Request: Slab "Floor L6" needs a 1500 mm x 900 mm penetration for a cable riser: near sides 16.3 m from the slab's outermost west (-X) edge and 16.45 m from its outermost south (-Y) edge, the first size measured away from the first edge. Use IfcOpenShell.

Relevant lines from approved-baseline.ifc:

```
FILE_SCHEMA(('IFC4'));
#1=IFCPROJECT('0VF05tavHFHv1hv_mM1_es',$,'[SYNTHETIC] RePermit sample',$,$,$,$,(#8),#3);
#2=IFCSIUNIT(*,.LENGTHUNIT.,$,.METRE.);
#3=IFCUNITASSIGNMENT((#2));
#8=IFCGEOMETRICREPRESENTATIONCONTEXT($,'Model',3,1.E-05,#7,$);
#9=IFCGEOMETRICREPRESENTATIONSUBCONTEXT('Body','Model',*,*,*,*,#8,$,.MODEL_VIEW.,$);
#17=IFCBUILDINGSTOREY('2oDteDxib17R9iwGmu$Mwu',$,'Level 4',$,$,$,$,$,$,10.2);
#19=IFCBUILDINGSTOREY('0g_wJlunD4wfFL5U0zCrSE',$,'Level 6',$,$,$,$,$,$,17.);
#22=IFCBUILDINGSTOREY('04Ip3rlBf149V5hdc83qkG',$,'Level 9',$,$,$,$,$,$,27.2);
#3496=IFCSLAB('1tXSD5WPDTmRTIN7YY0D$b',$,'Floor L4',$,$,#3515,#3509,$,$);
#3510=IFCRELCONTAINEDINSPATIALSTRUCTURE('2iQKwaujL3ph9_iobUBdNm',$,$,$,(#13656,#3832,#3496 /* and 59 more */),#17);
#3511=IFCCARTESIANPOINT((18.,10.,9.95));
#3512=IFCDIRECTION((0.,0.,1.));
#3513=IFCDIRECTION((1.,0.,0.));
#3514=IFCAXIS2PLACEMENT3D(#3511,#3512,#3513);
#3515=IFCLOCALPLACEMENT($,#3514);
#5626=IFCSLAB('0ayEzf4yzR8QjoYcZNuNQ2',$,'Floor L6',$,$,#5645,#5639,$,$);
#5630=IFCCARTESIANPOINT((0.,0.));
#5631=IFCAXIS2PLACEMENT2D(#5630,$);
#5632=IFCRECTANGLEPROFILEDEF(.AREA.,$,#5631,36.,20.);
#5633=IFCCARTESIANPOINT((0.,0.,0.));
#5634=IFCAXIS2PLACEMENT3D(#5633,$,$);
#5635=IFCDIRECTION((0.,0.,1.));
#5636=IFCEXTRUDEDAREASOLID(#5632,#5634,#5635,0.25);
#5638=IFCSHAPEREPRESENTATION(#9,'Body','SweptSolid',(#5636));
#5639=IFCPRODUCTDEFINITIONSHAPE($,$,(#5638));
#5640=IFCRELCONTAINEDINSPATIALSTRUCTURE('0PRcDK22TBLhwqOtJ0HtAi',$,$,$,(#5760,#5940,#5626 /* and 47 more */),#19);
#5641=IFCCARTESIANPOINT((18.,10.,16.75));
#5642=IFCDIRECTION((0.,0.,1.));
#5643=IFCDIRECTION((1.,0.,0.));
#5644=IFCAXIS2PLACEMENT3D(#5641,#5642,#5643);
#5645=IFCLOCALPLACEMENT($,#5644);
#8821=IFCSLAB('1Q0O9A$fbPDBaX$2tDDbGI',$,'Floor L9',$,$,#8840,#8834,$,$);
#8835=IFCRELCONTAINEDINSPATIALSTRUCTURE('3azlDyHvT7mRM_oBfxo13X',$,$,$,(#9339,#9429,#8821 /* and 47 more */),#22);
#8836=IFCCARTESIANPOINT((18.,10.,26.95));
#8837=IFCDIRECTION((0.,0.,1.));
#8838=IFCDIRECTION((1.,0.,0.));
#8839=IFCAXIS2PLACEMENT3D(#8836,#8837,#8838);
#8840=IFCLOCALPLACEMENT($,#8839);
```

```python
import numpy as np
import ifcopenshell
import ifcopenshell.api.feature
import ifcopenshell.api.geometry
import ifcopenshell.api.root
import ifcopenshell.geom
import ifcopenshell.util.placement
import ifcopenshell.util.representation
import ifcopenshell.util.shape
import ifcopenshell.util.unit

model = ifcopenshell.open("approved-baseline.ifc")
unit_scale = ifcopenshell.util.unit.calculate_unit_scale(model)
settings = ifcopenshell.geom.settings()


def volume(element):
    """Net volume in cubic metres, openings subtracted."""
    shape = ifcopenshell.geom.create_shape(settings, element)
    return ifcopenshell.util.shape.get_volume(shape.geometry)


slab = model.by_id(5626)
before = volume(slab)

# Extent in the slab's own axes, in metres. The edges named are its -X and -Y sides.
slab_shape = ifcopenshell.geom.create_shape(settings, slab)
vertices = ifcopenshell.util.shape.get_vertices(slab_shape.geometry)
x_min, y_min, bottom = vertices.min(axis=0)
top = vertices[:, 2].max()

opening = ifcopenshell.api.root.create_entity(model, ifc_class="IfcOpeningElement", name="Cable riser opening", predefined_type="OPENING")
context = ifcopenshell.util.representation.get_context(model, "Model", "Body", "MODEL_VIEW")
width, depth = 1.5, 0.9
outline = [(0.0, 0.0), (width, 0.0), (width, depth), (0.0, depth), (0.0, 0.0)]
# Overshoot both faces by 50 mm so the cut is clean.
shape = ifcopenshell.api.geometry.add_slab_representation(
    model, context=context, depth=top - bottom + 0.1, polyline=outline
)
ifcopenshell.api.geometry.assign_representation(model, product=opening, representation=shape)

matrix = ifcopenshell.util.placement.get_local_placement(slab.ObjectPlacement)
matrix[:, 3] = matrix @ np.append(np.array([x_min + 16.3, y_min + 16.45, bottom - 0.05]) / unit_scale, 1.0)
ifcopenshell.api.geometry.edit_object_placement(model, product=opening, matrix=matrix, is_si=False)
ifcopenshell.api.feature.add_feature(model, feature=opening, element=slab)

after = volume(slab)

print(f"slab volume {before:.3f} -> {after:.3f} m3")

model.write("approved-baseline_rev.ifc")
```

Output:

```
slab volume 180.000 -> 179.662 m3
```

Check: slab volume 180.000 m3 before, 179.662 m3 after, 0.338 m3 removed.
